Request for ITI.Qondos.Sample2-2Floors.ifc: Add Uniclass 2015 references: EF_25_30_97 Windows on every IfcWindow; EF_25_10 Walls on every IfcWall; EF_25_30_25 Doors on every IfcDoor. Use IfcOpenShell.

First a look at what the model holds.

```python
import ifcopenshell

model = ifcopenshell.open("ITI.Qondos.Sample2-2Floors.ifc")
print(model.schema)
print("classifications:", [c.Name for c in model.by_type("IfcClassification")])
for ifc_class in ("IfcDoor", "IfcRoof", "IfcStair", "IfcWall", "IfcWindow"):
    print(ifc_class, len(model.by_type(ifc_class)))
```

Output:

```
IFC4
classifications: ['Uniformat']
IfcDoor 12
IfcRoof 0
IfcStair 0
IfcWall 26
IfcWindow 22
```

```python
import ifcopenshell
import ifcopenshell.api.classification

model = ifcopenshell.open("ITI.Qondos.Sample2-2Floors.ifc")

system = ifcopenshell.api.classification.add_classification(model, classification="Uniclass 2015")

codes = {
    "IfcWindow": ("EF_25_30_97", "Windows"),
    "IfcWall": ("EF_25_10", "Walls"),
    "IfcDoor": ("EF_25_30_25", "Doors"),
}
for ifc_class, (code, name) in codes.items():
    products = model.by_type(ifc_class)
    ifcopenshell.api.classification.add_reference(
        model, products=products, classification=system, identification=code, name=name
    )
    print(code, len(products))

model.write("ITI.Qondos.Sample2-2Floors-out.ifc")
```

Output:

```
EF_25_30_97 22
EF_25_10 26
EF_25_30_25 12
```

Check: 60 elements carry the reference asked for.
